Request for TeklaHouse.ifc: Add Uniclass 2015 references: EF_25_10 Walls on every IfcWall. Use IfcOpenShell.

First a look at what the model holds.

```python
import ifcopenshell

model = ifcopenshell.open("TeklaHouse.ifc")
print(model.schema)
print("classifications:", [c.Name for c in model.by_type("IfcClassification")])
for ifc_class in ("IfcDoor", "IfcRoof", "IfcStair", "IfcWall", "IfcWindow"):
    print(ifc_class, len(model.by_type(ifc_class)))
```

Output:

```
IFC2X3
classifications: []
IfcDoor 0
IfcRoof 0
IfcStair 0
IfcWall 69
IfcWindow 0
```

```python
import ifcopenshell
import ifcopenshell.api.classification

model = ifcopenshell.open("TeklaHouse.ifc")

# IFC2X3 requires Source and Edition and has no link from the project to the system.
system = model.create_entity("IfcClassification", Source="NBS", Edition="2015", Name="Uniclass 2015")

codes = {
    "IfcWall": ("EF_25_10", "Walls"),
}
for ifc_class, (code, name) in codes.items():
    products = model.by_type(ifc_class)
    ifcopenshell.api.classification.add_reference(
        model, products=products, classification=system, identification=code, name=name
    )
    print(code, len(products))

model.write("TeklaHouse-out.ifc")
```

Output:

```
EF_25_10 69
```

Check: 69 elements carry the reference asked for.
